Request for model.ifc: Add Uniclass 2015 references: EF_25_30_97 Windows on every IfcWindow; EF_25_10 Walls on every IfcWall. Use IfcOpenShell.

First a look at what the model holds.

```python
import ifcopenshell

model = ifcopenshell.open("model.ifc")
print(model.schema)
print("classifications:", [c.Name for c in model.by_type("IfcClassification")])
for ifc_class in ("IfcDoor", "IfcRoof", "IfcStair", "IfcWall", "IfcWindow"):
    print(ifc_class, len(model.by_type(ifc_class)))
```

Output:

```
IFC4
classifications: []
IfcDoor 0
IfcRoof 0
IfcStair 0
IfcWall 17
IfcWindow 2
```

```python
import ifcopenshell
import ifcopenshell.api.classification

model = ifcopenshell.open("model.ifc")

system = ifcopenshell.api.classification.add_classification(model, classification="Uniclass 2015")

codes = {
    "IfcWindow": ("EF_25_30_97", "Windows"),
    "IfcWall": ("EF_25_10", "Walls"),
}
for ifc_class, (code, name) in codes.items():
    products = model.by_type(ifc_class)
    ifcopenshell.api.classification.add_reference(
        model, products=products, classification=system, identification=code, name=name
    )
    print(code, len(products))

model.write("model_edited.ifc")
```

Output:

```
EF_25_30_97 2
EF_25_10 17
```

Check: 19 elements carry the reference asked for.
